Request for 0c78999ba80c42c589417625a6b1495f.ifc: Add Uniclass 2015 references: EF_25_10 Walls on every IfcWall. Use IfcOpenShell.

First a look at what the model holds.

```python
import ifcopenshell

model = ifcopenshell.open("0c78999ba80c42c589417625a6b1495f.ifc")
print(model.schema)
print("classifications:", [c.Name for c in model.by_type("IfcClassification")])
for ifc_class in ("IfcDoor", "IfcRoof", "IfcStair", "IfcWall", "IfcWindow"):
    print(ifc_class, len(model.by_type(ifc_class)))
```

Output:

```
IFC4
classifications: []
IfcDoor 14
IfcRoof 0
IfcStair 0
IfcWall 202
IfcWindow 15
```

```python
import ifcopenshell
import ifcopenshell.api.classification

model = ifcopenshell.open("0c78999ba80c42c589417625a6b1495f.ifc")

system = ifcopenshell.api.classification.add_classification(model, classification="Uniclass 2015")

codes = {
    "IfcWall": ("EF_25_10", "Walls"),
}
for ifc_class, (code, name) in codes.items():
    products = model.by_type(ifc_class)
    ifcopenshell.api.classification.add_reference(
        model, products=products, classification=system, identification=code, name=name
    )
    print(code, len(products))

model.write("0c78999ba80c42c589417625a6b1495f_v2.ifc")
```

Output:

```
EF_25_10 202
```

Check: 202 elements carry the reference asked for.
